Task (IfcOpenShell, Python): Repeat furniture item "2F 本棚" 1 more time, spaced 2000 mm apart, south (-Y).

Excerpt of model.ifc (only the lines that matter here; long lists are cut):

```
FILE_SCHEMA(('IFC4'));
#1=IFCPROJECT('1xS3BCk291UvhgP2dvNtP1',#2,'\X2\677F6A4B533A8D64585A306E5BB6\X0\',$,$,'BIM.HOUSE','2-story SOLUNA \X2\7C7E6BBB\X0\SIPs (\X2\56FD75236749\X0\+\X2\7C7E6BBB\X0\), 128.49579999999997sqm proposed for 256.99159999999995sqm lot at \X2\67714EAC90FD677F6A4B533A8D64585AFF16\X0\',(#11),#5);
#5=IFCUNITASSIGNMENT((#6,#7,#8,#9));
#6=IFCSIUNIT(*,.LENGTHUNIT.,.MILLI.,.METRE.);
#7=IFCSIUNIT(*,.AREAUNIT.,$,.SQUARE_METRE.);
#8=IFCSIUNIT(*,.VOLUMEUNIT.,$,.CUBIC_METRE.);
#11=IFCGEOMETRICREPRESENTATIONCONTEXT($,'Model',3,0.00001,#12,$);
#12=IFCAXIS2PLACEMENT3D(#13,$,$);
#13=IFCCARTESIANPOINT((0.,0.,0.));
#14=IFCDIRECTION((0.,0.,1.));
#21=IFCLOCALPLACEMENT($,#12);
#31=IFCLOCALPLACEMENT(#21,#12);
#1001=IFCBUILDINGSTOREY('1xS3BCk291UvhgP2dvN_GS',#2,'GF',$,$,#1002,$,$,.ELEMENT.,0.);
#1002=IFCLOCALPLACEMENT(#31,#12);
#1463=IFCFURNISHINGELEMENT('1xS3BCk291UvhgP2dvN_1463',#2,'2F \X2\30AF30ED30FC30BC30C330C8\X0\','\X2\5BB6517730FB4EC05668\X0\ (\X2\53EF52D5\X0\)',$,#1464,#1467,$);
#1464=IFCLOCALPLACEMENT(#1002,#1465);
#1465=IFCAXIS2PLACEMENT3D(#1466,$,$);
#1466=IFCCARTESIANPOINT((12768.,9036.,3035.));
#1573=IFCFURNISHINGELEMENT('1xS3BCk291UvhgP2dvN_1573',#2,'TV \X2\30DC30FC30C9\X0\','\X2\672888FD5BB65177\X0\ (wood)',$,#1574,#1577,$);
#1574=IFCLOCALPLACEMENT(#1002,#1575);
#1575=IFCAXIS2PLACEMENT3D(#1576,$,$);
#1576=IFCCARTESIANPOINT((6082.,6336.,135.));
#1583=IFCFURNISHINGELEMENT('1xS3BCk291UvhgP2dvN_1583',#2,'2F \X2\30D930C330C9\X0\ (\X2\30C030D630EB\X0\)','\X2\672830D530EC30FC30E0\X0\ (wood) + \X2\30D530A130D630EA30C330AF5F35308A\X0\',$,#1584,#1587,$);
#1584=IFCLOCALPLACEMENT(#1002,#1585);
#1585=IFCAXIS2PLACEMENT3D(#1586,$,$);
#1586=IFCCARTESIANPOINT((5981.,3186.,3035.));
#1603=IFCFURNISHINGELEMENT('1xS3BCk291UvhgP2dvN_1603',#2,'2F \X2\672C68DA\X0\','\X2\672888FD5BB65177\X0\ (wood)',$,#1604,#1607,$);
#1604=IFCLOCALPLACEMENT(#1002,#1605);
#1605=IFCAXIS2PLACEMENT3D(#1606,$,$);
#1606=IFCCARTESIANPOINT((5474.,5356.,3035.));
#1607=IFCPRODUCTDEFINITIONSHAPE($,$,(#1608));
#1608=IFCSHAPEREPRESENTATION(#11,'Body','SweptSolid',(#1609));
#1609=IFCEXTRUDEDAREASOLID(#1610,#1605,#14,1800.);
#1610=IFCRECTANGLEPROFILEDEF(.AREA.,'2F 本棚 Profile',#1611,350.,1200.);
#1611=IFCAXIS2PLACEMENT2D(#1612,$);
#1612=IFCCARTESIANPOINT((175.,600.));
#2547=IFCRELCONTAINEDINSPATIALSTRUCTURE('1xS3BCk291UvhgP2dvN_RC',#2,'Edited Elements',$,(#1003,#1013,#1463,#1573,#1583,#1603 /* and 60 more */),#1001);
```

```python
import numpy as np
import ifcopenshell
import ifcopenshell.api.geometry
import ifcopenshell.api.root
import ifcopenshell.util.element
import ifcopenshell.util.placement

model = ifcopenshell.open("model.ifc")


def reuse_history(source, copy):
    """copy_class also copies each property set's owner history, people and application; keep the originals."""
    for rel in copy.IsDefinedBy:
        if rel.is_a("IfcRelDefinesByProperties") and (history := rel.RelatingPropertyDefinition.OwnerHistory):
            rel.RelatingPropertyDefinition.OwnerHistory = source.OwnerHistory
            ifcopenshell.util.element.remove_deep2(model, history)


source = model.by_guid("1xS3BCk291UvhgP2dvN_1603")
base = ifcopenshell.util.placement.get_local_placement(source.ObjectPlacement)
step = np.array([0.0, -1.0, 0.0]) * 2000.0

for i in range(1, 2):
    copy = ifcopenshell.api.root.copy_class(model, product=source)
    copy.Representation = ifcopenshell.util.element.copy_deep(
        model, source.Representation, exclude=["IfcGeometricRepresentationContext", "IfcRepresentationMap"]
    )
    reuse_history(source, copy)
    matrix = base.copy()
    matrix[:3, 3] += i * step
    print("added at", matrix[:3, 3].round(3) + 0.0)
    ifcopenshell.api.geometry.edit_object_placement(model, product=copy, matrix=matrix, is_si=False)

model.write("model_updated.ifc")
```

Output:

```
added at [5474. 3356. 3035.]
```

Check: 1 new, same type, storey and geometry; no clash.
